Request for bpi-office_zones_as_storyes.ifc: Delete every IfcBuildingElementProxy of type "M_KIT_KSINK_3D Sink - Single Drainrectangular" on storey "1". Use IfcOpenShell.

First a look at what the model holds.

```python
import ifcopenshell
import ifcopenshell.util.element

model = ifcopenshell.open("bpi-office_zones_as_storyes.ifc")
print(model.schema)
storey = next(s for s in model.by_type("IfcBuildingStorey") if s.Name == "1")
proxies = [e for e in ifcopenshell.util.element.get_decomposition(storey) if e.is_a("IfcBuildingElementProxy")]
seen = {}
for e in proxies:
    element_type = ifcopenshell.util.element.get_type(e)
    name = element_type.Name if element_type not in (None, e) else None
    seen[name] = seen.get(name, 0) + 1
for name, count in sorted(seen.items(), key=str):
    print(count, "x", name)
```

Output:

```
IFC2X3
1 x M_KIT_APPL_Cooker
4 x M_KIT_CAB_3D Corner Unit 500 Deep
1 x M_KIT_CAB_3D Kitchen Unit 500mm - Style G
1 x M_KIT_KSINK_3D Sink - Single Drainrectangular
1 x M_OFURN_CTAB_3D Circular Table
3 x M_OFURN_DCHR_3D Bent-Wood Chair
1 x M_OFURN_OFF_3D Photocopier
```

```python
import ifcopenshell
import ifcopenshell.api.root
import ifcopenshell.util.element

model = ifcopenshell.open("bpi-office_zones_as_storyes.ifc")

storey = next(s for s in model.by_type("IfcBuildingStorey") if s.Name == "1")
proxies = [e for e in ifcopenshell.util.element.get_decomposition(storey) if e.is_a("IfcBuildingElementProxy")]
targets = [e for e in proxies if (t := ifcopenshell.util.element.get_type(e)) not in (None, e) and t.Name == "M_KIT_KSINK_3D Sink - Single Drainrectangular"]

for e in targets:
    ifcopenshell.api.root.remove_product(model, product=e)
print(len(targets), "removed")

model.write("bpi-office_zones_as_storyes_v2.ifc")
```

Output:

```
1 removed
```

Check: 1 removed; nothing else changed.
